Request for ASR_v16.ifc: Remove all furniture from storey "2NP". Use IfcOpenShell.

First a look at what the model holds.

```python
import ifcopenshell
import ifcopenshell.util.element

model = ifcopenshell.open("ASR_v16.ifc")
print(model.schema)
storey = next(s for s in model.by_type("IfcBuildingStorey") if s.Name == "2NP")
furniture = [e for e in ifcopenshell.util.element.get_decomposition(storey) if e.is_a("IfcFurnishingElement")]
seen = {}
for e in furniture:
    element_type = ifcopenshell.util.element.get_type(e)
    name = element_type.Name if element_type not in (None, e) else None
    seen[name] = seen.get(name, 0) + 1
for name, count in sorted(seen.items(), key=str):
    print(count, "x", name)
```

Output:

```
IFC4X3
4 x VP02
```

```python
import ifcopenshell
import ifcopenshell.api.root
import ifcopenshell.util.element

model = ifcopenshell.open("ASR_v16.ifc")

storey = next(s for s in model.by_type("IfcBuildingStorey") if s.Name == "2NP")
furniture = [e for e in ifcopenshell.util.element.get_decomposition(storey) if e.is_a("IfcFurnishingElement")]

for e in furniture:
    ifcopenshell.api.root.remove_product(model, product=e)
print(len(furniture), "removed")

model.write("ASR_v16_v2.ifc")
```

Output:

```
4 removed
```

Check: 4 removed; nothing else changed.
